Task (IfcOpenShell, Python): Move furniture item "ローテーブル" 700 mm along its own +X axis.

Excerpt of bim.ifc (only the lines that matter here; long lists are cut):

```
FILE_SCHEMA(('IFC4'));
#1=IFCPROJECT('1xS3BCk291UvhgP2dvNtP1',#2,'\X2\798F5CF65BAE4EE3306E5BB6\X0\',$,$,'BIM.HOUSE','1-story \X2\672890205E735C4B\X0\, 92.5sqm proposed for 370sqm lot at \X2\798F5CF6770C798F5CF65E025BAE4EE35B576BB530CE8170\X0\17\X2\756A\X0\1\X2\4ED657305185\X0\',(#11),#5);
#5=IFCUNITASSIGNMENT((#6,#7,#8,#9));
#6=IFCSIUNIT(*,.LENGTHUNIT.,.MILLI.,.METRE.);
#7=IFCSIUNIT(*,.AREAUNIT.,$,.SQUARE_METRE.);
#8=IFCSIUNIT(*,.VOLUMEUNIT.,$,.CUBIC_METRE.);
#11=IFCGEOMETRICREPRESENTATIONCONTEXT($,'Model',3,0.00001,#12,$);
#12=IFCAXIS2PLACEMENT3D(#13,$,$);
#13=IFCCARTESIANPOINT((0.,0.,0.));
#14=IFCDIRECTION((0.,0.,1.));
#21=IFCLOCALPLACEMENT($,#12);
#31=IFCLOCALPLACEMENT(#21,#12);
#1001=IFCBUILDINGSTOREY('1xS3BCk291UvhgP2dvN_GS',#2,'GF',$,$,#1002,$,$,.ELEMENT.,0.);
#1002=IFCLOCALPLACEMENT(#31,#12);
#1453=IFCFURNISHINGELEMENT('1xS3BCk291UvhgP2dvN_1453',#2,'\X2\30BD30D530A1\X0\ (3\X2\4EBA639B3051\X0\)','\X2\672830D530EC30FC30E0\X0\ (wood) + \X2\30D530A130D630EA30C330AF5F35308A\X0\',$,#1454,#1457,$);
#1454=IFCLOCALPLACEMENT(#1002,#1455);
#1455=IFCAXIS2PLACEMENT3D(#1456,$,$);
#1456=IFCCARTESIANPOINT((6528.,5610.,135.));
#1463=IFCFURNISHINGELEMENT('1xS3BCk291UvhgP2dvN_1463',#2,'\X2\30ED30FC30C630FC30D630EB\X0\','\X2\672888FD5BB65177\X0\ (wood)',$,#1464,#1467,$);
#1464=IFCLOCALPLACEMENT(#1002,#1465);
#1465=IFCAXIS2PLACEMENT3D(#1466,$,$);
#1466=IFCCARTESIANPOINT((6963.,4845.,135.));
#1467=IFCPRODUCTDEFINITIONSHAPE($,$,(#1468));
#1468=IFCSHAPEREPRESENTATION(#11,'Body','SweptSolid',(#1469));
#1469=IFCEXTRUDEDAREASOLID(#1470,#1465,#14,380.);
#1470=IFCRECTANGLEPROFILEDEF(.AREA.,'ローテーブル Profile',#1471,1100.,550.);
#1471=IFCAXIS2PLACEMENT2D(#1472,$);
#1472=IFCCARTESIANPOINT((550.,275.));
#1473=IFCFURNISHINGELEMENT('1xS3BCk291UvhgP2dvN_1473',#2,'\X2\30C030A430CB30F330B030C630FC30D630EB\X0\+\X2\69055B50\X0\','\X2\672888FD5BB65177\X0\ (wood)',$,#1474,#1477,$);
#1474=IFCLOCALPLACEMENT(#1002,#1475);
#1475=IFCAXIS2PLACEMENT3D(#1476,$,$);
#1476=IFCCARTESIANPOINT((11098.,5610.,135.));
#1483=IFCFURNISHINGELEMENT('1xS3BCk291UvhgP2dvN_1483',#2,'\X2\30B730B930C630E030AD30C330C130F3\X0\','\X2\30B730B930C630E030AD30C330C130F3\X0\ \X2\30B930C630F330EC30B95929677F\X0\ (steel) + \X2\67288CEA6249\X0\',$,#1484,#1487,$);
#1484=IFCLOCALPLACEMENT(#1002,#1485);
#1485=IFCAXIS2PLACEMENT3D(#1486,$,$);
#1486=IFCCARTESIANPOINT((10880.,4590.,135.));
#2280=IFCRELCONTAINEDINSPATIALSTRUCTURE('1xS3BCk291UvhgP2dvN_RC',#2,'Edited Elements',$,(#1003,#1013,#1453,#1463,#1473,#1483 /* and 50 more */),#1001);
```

```python
import ifcopenshell
import ifcopenshell.api.geometry
import ifcopenshell.util.placement

model = ifcopenshell.open("bim.ifc")

item = model.by_id(1463)
matrix = ifcopenshell.util.placement.get_local_placement(item.ObjectPlacement)
matrix[:3, 3] += matrix[:3, 0] * 700.0
ifcopenshell.api.geometry.edit_object_placement(model, product=item, matrix=matrix, is_si=False)

print(ifcopenshell.util.placement.get_local_placement(item.ObjectPlacement).round(3) + 0.0)

model.write("bim_rev.ifc")
```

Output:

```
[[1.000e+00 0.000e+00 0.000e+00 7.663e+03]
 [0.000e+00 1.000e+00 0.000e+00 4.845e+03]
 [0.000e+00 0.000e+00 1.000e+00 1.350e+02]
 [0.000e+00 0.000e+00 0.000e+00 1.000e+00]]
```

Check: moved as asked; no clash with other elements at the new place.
